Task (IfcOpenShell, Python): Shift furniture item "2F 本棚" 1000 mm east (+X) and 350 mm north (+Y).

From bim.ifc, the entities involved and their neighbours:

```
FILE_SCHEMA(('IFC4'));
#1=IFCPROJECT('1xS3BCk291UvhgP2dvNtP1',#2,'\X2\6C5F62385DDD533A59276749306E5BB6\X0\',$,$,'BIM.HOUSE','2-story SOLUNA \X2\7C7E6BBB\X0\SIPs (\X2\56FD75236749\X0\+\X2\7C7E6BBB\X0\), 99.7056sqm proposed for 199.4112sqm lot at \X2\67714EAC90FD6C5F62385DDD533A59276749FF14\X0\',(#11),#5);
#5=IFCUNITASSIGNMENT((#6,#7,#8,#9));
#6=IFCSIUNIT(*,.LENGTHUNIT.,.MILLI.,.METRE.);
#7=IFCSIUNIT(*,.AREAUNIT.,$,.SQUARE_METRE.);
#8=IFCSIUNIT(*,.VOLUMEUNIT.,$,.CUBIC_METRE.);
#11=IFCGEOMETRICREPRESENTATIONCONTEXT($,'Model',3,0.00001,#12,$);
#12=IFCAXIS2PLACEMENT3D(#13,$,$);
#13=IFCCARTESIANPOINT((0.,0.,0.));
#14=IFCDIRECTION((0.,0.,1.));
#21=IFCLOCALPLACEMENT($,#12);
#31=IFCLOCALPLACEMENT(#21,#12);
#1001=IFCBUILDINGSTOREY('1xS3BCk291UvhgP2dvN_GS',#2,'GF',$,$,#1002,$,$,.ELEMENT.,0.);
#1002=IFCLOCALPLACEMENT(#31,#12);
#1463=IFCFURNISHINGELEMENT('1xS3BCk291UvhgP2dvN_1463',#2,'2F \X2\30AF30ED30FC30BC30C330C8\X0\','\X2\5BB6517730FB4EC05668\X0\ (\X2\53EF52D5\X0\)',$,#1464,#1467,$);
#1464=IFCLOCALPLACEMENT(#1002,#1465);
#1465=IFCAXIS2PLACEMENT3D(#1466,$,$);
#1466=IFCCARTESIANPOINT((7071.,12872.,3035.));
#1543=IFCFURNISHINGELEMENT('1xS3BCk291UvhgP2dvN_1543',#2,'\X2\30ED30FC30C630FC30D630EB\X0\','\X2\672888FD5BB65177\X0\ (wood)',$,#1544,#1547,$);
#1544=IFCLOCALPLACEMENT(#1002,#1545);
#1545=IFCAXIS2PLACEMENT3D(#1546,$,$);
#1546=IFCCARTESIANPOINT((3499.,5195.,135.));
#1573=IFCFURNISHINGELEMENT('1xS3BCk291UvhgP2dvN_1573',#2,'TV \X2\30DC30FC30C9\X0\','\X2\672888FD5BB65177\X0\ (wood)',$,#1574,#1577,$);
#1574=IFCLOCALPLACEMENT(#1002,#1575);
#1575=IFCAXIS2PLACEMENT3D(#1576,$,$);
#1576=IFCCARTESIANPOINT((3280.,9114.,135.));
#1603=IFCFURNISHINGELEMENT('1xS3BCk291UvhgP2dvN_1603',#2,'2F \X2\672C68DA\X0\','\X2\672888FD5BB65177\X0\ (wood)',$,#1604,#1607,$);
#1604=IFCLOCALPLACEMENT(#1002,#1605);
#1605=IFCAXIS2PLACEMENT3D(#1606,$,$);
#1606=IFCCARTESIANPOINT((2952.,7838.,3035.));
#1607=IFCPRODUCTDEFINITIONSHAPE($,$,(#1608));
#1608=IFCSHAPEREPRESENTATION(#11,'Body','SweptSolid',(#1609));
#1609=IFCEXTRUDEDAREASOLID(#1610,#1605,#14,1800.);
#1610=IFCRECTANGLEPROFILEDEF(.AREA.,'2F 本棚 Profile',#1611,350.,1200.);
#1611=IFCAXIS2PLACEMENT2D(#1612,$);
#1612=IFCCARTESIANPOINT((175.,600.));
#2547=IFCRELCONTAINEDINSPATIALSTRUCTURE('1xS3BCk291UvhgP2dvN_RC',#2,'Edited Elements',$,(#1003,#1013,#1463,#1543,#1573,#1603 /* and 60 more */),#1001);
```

```python
import ifcopenshell
import ifcopenshell.api.geometry
import ifcopenshell.util.placement

model = ifcopenshell.open("bim.ifc")

item = model.by_guid("1xS3BCk291UvhgP2dvN_1603")
matrix = ifcopenshell.util.placement.get_local_placement(item.ObjectPlacement)
matrix[0, 3] += 1000.0
matrix[1, 3] += 350.0
ifcopenshell.api.geometry.edit_object_placement(model, product=item, matrix=matrix, is_si=False)

print(ifcopenshell.util.placement.get_local_placement(item.ObjectPlacement).round(3) + 0.0)

model.write("bim_v2.ifc")
```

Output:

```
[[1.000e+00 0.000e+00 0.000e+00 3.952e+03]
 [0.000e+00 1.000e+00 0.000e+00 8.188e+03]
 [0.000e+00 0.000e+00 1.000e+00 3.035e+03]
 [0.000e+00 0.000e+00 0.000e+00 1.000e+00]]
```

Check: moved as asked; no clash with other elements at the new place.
